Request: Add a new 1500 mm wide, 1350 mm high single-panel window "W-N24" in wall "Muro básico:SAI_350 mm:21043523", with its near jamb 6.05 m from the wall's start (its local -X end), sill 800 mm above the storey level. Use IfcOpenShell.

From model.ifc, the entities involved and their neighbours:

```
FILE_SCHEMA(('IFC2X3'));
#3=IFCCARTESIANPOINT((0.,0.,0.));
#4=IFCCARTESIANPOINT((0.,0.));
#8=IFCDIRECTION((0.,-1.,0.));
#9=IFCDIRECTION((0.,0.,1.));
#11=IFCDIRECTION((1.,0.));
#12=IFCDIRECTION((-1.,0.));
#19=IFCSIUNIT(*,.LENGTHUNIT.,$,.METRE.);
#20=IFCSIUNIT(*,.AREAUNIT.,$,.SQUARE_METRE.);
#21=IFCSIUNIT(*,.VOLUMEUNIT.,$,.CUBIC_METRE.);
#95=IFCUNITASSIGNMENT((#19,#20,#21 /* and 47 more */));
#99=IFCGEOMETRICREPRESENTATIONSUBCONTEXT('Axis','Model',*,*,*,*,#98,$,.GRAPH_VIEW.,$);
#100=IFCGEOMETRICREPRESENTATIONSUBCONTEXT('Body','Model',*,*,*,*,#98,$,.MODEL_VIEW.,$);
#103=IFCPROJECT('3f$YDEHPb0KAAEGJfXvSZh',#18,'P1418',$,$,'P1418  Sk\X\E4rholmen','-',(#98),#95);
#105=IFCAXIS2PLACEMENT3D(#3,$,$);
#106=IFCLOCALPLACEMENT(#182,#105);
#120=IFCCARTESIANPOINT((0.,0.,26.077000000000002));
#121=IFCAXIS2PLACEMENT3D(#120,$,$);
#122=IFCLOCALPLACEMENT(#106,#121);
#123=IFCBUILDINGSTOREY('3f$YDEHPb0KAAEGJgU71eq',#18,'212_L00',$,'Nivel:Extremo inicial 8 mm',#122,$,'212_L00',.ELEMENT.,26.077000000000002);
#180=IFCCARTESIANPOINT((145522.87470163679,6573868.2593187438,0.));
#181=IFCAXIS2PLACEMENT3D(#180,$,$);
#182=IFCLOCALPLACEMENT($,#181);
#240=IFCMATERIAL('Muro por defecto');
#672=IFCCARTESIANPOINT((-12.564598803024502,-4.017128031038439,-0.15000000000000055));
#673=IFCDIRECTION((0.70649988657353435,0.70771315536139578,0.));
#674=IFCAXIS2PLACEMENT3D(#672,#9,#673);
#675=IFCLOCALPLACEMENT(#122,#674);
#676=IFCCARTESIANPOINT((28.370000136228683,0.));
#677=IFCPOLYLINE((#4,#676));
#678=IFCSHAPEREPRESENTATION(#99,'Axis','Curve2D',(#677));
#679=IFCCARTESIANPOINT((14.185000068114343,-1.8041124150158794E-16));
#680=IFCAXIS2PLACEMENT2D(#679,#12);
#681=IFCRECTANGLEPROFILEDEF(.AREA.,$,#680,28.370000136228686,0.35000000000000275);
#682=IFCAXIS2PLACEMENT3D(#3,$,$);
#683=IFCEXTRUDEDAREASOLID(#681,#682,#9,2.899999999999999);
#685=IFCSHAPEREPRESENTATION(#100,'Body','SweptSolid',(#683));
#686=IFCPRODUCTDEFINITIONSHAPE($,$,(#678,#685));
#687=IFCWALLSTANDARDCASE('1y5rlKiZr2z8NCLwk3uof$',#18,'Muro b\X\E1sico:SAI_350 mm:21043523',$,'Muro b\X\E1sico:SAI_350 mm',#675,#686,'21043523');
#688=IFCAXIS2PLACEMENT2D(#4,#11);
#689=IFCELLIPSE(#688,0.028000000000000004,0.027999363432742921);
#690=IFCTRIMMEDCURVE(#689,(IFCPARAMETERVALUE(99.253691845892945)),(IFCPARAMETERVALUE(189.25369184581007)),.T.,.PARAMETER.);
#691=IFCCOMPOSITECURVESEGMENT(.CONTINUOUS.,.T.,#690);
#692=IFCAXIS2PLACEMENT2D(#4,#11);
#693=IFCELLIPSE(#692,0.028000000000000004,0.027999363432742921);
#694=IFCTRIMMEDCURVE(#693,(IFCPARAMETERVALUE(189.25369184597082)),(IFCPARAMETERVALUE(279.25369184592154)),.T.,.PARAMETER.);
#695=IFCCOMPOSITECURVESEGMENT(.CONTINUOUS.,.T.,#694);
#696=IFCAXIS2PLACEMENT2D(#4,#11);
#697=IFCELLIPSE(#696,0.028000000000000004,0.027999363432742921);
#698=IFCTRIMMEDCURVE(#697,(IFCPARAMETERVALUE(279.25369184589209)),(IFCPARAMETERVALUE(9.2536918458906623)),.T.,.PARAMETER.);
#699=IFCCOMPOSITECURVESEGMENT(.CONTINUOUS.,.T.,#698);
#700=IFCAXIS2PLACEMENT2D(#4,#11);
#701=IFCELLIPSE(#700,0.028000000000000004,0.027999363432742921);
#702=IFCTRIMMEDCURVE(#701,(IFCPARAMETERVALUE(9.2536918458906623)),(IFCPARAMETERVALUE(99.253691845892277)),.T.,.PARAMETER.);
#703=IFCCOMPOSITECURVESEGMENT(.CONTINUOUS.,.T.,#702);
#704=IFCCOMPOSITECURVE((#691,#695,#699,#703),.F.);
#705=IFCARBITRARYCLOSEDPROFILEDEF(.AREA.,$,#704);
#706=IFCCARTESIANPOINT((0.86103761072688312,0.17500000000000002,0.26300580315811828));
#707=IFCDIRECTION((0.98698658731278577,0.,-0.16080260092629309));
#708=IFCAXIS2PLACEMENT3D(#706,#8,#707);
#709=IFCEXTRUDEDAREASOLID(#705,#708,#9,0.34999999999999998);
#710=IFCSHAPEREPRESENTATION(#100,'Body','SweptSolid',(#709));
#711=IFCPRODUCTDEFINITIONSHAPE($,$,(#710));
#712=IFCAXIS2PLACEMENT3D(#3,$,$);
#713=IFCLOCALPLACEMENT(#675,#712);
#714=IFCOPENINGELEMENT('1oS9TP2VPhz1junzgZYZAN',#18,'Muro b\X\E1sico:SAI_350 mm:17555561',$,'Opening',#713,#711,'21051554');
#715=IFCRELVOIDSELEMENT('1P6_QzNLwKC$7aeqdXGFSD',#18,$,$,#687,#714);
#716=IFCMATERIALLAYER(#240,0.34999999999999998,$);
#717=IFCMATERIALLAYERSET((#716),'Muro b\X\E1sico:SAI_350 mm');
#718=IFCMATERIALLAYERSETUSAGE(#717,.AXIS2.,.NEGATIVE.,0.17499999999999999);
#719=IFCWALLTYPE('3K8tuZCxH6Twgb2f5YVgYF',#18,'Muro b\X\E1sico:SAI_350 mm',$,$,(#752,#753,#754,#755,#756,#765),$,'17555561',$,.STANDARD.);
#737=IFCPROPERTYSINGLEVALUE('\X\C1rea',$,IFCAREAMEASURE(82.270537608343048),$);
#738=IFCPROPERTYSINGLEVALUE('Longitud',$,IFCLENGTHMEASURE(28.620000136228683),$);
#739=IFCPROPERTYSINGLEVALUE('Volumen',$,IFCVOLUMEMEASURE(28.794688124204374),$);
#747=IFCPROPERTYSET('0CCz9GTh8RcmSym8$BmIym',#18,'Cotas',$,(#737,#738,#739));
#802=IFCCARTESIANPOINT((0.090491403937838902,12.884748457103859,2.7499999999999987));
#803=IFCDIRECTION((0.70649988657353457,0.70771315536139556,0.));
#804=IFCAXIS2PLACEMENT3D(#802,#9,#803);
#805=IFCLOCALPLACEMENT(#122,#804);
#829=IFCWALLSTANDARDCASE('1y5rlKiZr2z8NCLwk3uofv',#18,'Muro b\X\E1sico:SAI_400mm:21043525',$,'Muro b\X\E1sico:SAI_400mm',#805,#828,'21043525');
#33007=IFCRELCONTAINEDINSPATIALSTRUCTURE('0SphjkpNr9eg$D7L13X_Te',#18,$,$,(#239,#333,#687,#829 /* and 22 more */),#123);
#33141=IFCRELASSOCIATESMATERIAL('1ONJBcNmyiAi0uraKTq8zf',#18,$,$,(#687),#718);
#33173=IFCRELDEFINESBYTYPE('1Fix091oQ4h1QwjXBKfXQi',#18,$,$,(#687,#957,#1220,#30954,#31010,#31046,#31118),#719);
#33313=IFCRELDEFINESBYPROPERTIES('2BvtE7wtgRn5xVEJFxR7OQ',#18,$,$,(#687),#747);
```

```python
import numpy as np
import ifcopenshell
import ifcopenshell.api.feature
import ifcopenshell.api.geometry
import ifcopenshell.api.pset
import ifcopenshell.api.root
import ifcopenshell.api.spatial
import ifcopenshell.api.type
import ifcopenshell.geom
import ifcopenshell.util.element
import ifcopenshell.util.placement
import ifcopenshell.util.representation
import ifcopenshell.util.shape
import ifcopenshell.util.unit

model = ifcopenshell.open("model.ifc")
unit_scale = ifcopenshell.util.unit.calculate_unit_scale(model)
area_scale = ifcopenshell.util.unit.calculate_unit_scale(model, "AREAUNIT")
volume_scale = ifcopenshell.util.unit.calculate_unit_scale(model, "VOLUMEUNIT")
settings = ifcopenshell.geom.settings()


def volume(element):
    """Net volume in cubic metres, openings subtracted."""
    shape = ifcopenshell.geom.create_shape(settings, element)
    return ifcopenshell.util.shape.get_volume(shape.geometry)


wall = model.by_id(687)
storey = ifcopenshell.util.element.get_container(wall, ifc_class="IfcBuildingStorey")
context = ifcopenshell.util.representation.get_context(model, "Model", "Body", "MODEL_VIEW")
before = volume(wall)

width, height, from_end, sill = 1.5, 1.35, 6.05, 0.8  # metres

# The wall runs along its own X axis, and the end named is its -X end.
wall_shape = ifcopenshell.geom.create_shape(settings, wall)
x, y, z = ifcopenshell.util.shape.get_vertices(wall_shape.geometry).T
start = x.min() + from_end
face, thickness = float(y.min()), float(y.max() - y.min())
wall_matrix = ifcopenshell.util.placement.get_local_placement(wall.ObjectPlacement)
level = ifcopenshell.util.placement.get_local_placement(storey.ObjectPlacement)[2, 3]


def in_wall(x, y):
    """Placement at x, y metres in the wall's axes, at sill height."""
    matrix = wall_matrix.copy()
    matrix[:, 3] = wall_matrix @ np.array([x / unit_scale, y / unit_scale, 0.0, 1.0])
    matrix[2, 3] = level + sill / unit_scale
    return matrix


# Opening: a box that overshoots both wall faces by 50 mm.
opening = ifcopenshell.api.root.create_entity(model, ifc_class="IfcOpeningElement")
box = ifcopenshell.api.geometry.add_wall_representation(
    model, context=context, length=width, height=height, thickness=thickness + 0.1
)
ifcopenshell.api.geometry.assign_representation(model, product=opening, representation=box)
ifcopenshell.api.geometry.edit_object_placement(model, product=opening, matrix=in_wall(start, face - 0.05), is_si=False)
ifcopenshell.api.feature.add_feature(model, feature=opening, element=wall)

window = ifcopenshell.api.root.create_entity(model, ifc_class="IfcWindow", name="W-N24")
window.OverallWidth, window.OverallHeight = width / unit_scale, height / unit_scale
body = ifcopenshell.api.geometry.add_window_representation(
    model,
    context=context,
    overall_width=window.OverallWidth,
    overall_height=window.OverallHeight,
    partition_type="SINGLE_PANEL",
)
ifcopenshell.api.geometry.assign_representation(model, product=window, representation=body)
ifcopenshell.api.spatial.assign_container(model, products=[window], relating_structure=storey)
fills = ifcopenshell.api.feature.add_filling(model, opening=opening, element=window)
fills.OwnerHistory = window.OwnerHistory  # required in IFC2X3

# IFC2X3 keeps the operation on the window style.
style = ifcopenshell.api.root.create_entity(model, ifc_class="IfcWindowStyle", name="W-N24")
style.OperationType, style.ConstructionType = "SINGLE_PANEL", "NOTDEFINED"
style.ParameterTakesPrecedence = style.Sizeable = False
ifcopenshell.api.type.assign_type(model, related_objects=[window], relating_type=style)

# Centre the window in the wall's thickness.
ifcopenshell.api.geometry.edit_object_placement(model, product=window, matrix=in_wall(start, face), is_si=False)
window_shape = ifcopenshell.geom.create_shape(settings, window)
depth = ifcopenshell.util.shape.get_vertices(window_shape.geometry)[:, 1]
offset = face + thickness / 2 - (depth.min() + depth.max()) / 2
ifcopenshell.api.geometry.edit_object_placement(model, product=window, matrix=in_wall(start, offset), is_si=False)

after = volume(wall)

# Update the wall's stored quantities.
pset = model.by_id(ifcopenshell.util.element.get_pset(wall, "Cotas", should_inherit=False)["id"])
ifcopenshell.api.pset.edit_pset(model, pset=pset, properties={
    "Área": model.create_entity("IfcAreaMeasure", after / thickness / area_scale),
    "Volumen": model.create_entity("IfcVolumeMeasure", after / volume_scale),
})

print(f"wall volume {before:.3f} -> {after:.3f} m3")

model.write("model-out.ifc")
```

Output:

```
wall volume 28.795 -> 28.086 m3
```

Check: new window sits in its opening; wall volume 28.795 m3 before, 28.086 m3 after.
